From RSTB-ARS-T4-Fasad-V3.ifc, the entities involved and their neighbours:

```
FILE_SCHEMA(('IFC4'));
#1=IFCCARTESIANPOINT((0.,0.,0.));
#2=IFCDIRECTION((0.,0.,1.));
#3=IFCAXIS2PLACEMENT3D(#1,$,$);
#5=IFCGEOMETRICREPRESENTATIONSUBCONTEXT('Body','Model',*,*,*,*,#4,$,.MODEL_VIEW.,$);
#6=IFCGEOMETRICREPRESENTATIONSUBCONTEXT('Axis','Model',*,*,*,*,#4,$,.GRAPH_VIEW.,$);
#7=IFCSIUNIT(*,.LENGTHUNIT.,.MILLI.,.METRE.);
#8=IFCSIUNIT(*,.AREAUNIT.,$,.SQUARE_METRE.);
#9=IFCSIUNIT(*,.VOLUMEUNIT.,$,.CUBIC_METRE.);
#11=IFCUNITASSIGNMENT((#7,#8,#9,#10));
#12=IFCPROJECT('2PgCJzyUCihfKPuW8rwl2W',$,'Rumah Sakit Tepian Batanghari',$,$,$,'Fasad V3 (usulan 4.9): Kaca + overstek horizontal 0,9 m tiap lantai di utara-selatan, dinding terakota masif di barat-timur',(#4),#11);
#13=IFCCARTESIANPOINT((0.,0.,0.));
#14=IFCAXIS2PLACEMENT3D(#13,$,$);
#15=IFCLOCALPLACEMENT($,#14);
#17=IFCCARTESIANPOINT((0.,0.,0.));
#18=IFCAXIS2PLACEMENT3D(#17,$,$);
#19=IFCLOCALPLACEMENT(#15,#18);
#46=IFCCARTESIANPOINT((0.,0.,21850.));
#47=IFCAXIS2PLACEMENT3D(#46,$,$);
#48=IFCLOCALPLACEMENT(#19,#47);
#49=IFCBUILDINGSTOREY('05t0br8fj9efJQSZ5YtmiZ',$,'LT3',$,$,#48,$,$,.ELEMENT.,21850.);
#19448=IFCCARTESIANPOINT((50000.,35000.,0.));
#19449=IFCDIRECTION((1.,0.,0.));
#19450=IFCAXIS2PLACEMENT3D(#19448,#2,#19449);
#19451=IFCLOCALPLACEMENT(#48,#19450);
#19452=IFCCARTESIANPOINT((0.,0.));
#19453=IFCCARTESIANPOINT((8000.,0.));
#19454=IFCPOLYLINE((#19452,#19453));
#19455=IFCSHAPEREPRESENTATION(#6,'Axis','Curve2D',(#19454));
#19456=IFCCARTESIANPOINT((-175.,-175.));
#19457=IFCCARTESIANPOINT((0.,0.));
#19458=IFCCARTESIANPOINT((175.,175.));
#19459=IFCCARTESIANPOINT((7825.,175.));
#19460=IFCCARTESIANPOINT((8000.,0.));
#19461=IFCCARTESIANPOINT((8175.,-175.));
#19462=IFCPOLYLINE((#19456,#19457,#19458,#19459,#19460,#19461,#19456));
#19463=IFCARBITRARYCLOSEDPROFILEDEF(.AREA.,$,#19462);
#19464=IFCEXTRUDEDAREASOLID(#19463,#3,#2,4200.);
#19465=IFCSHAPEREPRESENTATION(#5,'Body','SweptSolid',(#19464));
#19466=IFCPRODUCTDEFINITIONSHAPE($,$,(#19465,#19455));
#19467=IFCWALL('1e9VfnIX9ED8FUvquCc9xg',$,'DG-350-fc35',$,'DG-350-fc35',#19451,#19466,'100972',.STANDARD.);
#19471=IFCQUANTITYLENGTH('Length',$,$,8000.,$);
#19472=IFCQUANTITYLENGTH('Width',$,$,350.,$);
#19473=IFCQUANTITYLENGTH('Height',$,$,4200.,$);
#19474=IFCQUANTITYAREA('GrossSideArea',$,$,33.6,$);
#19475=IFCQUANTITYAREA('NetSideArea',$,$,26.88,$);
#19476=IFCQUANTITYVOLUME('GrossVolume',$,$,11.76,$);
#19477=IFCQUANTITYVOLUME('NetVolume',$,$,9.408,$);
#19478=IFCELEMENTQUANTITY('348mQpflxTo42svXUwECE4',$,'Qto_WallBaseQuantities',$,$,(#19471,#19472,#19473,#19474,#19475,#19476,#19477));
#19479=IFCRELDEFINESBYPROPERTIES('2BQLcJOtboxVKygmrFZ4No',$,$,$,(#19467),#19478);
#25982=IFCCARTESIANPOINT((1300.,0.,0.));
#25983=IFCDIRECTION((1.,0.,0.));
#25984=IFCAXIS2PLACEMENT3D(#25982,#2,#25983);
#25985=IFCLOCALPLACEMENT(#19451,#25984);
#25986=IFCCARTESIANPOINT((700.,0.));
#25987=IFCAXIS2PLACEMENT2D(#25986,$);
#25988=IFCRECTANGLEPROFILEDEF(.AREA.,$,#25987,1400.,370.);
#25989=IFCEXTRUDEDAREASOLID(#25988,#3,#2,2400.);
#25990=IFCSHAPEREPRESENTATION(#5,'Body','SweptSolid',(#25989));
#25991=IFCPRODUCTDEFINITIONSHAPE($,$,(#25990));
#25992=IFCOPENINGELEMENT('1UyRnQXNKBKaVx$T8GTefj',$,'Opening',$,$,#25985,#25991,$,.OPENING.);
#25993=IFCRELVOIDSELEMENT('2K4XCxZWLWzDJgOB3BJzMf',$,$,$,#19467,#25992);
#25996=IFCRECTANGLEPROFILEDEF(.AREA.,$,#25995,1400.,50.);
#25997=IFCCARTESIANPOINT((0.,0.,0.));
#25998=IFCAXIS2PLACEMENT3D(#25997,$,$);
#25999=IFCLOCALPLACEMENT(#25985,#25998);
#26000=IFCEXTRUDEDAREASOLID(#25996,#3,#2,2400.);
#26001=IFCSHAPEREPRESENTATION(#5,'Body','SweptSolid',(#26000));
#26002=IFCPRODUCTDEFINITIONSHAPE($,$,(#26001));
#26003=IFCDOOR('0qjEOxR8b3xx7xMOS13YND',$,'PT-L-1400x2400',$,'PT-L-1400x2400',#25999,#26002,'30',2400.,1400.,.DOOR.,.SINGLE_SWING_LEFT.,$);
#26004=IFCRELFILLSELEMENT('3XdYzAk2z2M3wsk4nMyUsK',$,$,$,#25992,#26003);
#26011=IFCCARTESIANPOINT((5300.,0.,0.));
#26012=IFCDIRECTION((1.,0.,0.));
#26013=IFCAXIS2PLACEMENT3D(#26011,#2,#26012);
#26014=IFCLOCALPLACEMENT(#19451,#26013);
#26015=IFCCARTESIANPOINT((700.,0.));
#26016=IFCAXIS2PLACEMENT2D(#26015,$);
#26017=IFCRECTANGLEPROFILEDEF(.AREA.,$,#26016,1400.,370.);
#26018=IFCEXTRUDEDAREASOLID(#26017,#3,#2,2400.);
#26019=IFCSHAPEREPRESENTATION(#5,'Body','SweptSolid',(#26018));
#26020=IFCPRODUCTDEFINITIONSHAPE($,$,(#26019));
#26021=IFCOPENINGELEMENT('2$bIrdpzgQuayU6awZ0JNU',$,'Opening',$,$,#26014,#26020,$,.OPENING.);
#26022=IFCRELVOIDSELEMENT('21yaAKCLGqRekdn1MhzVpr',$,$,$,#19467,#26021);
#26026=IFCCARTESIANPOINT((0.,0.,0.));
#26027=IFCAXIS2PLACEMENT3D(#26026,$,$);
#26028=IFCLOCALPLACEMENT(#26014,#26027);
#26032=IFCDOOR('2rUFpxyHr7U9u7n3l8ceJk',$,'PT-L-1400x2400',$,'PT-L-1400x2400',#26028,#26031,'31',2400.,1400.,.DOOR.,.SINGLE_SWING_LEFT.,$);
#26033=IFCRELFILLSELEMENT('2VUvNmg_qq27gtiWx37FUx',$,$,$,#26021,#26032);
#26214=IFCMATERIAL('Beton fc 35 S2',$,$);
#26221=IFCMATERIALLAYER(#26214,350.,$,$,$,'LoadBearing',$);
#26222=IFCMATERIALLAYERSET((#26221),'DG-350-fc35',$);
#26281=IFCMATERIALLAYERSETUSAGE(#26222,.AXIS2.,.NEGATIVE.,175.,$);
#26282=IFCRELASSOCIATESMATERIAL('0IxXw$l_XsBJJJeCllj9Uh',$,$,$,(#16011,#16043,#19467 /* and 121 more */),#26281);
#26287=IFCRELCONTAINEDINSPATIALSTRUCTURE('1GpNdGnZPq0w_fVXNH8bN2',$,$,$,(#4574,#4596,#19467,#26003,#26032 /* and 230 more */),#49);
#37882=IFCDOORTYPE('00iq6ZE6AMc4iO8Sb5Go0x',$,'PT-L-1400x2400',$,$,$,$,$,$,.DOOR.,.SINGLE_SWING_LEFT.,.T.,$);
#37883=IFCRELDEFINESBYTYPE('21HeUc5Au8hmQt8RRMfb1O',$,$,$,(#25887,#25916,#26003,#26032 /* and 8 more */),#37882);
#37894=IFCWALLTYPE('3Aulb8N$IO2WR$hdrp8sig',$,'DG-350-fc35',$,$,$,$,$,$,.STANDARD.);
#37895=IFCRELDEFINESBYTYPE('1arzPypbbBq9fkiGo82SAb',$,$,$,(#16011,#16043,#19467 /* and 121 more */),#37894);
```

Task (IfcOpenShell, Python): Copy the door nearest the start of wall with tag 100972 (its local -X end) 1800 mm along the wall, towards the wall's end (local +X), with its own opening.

```python
import ifcopenshell
import ifcopenshell.api.feature
import ifcopenshell.api.geometry
import ifcopenshell.api.pset
import ifcopenshell.api.root
import ifcopenshell.geom
import ifcopenshell.util.element
import ifcopenshell.util.placement
import ifcopenshell.util.shape
import ifcopenshell.util.unit

model = ifcopenshell.open("RSTB-ARS-T4-Fasad-V3.ifc")
area_scale = ifcopenshell.util.unit.calculate_unit_scale(model, "AREAUNIT")
volume_scale = ifcopenshell.util.unit.calculate_unit_scale(model, "VOLUMEUNIT")
settings = ifcopenshell.geom.settings()


def volume(element):
    """Net volume in cubic metres, openings subtracted."""
    shape = ifcopenshell.geom.create_shape(settings, element)
    return ifcopenshell.util.shape.get_volume(shape.geometry)


door = model.by_guid("0qjEOxR8b3xx7xMOS13YND")
opening = door.FillsVoids[0].RelatingOpeningElement
wall = opening.VoidsElements[0].RelatingBuildingElement
before = volume(wall)
shift = ifcopenshell.util.placement.get_local_placement(wall.ObjectPlacement)[:3, 0] * 1800.0

# copy_class copies the void relationship, type, container and properties, but no geometry.
new_opening = ifcopenshell.api.root.copy_class(model, product=opening)
new_opening.Representation = ifcopenshell.util.element.copy_deep(
    model, opening.Representation, exclude=["IfcGeometricRepresentationContext", "IfcRepresentationMap"]
)
new_door = ifcopenshell.api.root.copy_class(model, product=door)
new_door.Representation = ifcopenshell.util.element.copy_deep(
    model, door.Representation, exclude=["IfcGeometricRepresentationContext", "IfcRepresentationMap"]
)
new_door.Tag = None
ifcopenshell.api.feature.add_filling(model, opening=new_opening, element=new_door)

for old, new in ((opening, new_opening), (door, new_door)):
    matrix = ifcopenshell.util.placement.get_local_placement(old.ObjectPlacement)
    matrix[:3, 3] += shift
    ifcopenshell.api.geometry.edit_object_placement(model, product=new, matrix=matrix, is_si=False)

after = volume(wall)
thickness = 0.35  # wall thickness in metres

# Update the wall's stored quantities.
qto = model.by_id(ifcopenshell.util.element.get_pset(wall, "Qto_WallBaseQuantities", should_inherit=False)["id"])
ifcopenshell.api.pset.edit_qto(model, qto=qto, properties={
    "NetSideArea": after / thickness / area_scale,
    "NetVolume": after / volume_scale,
})

print(f"wall volume {before:.3f} -> {after:.3f} m3")

model.write("RSTB-ARS-T4-Fasad-V3_v2.ifc")
```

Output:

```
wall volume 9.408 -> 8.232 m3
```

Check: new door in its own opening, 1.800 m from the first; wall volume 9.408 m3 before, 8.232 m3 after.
